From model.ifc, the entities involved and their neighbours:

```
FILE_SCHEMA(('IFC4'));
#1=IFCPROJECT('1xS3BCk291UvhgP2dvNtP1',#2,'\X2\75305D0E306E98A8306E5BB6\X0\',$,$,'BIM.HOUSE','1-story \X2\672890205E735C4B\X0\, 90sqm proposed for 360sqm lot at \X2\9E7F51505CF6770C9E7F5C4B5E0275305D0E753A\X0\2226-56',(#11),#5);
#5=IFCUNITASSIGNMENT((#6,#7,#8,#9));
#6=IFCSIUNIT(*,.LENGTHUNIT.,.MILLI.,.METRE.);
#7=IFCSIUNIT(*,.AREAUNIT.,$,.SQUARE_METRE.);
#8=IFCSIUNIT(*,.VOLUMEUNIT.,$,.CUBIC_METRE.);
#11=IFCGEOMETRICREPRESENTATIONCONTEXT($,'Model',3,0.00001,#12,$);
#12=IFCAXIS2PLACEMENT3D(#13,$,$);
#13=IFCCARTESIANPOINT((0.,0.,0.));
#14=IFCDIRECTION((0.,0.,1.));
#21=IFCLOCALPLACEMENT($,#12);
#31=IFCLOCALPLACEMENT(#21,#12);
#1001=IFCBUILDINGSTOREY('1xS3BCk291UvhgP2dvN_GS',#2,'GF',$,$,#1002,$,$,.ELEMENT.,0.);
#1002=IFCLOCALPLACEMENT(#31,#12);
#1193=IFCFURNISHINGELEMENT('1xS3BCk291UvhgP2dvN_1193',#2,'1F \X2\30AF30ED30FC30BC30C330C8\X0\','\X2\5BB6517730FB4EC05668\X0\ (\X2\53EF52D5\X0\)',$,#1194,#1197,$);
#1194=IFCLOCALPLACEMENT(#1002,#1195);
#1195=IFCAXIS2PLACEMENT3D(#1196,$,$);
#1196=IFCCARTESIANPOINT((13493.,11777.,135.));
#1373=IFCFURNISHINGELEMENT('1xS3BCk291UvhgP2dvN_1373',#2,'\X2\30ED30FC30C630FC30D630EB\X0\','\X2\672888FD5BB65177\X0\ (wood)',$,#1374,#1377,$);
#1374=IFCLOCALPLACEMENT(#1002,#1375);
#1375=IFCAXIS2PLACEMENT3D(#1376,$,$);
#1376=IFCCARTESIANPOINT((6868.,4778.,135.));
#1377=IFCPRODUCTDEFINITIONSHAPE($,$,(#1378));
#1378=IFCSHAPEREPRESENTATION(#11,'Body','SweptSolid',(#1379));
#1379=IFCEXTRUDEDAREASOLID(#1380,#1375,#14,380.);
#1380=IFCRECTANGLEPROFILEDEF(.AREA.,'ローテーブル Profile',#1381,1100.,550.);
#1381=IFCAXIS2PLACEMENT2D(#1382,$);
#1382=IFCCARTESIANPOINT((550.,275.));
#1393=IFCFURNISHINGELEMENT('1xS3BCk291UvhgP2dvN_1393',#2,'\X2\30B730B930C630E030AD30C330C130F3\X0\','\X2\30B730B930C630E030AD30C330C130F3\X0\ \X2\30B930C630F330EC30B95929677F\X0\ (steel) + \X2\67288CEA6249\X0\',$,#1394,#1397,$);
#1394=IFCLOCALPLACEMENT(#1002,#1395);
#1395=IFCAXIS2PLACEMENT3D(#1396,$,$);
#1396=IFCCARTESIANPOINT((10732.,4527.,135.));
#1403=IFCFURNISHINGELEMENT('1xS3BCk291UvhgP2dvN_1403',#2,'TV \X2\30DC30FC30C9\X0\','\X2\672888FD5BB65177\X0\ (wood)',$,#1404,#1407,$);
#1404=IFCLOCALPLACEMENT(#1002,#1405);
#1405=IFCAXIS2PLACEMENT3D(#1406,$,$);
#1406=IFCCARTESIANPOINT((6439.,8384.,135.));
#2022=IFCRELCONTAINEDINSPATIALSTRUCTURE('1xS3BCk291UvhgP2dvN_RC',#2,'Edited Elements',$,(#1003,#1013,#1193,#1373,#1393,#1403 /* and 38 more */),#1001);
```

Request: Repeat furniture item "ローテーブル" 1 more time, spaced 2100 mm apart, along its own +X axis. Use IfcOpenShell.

```python
import ifcopenshell
import ifcopenshell.api.geometry
import ifcopenshell.api.root
import ifcopenshell.util.element
import ifcopenshell.util.placement
import ifcopenshell.util.unit

model = ifcopenshell.open("model.ifc")
unit_scale = ifcopenshell.util.unit.calculate_unit_scale(model)


def reuse_history(source, copy):
    """copy_class also copies each property set's owner history, people and application; keep the originals."""
    for rel in copy.IsDefinedBy:
        if rel.is_a("IfcRelDefinesByProperties") and (history := rel.RelatingPropertyDefinition.OwnerHistory):
            rel.RelatingPropertyDefinition.OwnerHistory = source.OwnerHistory
            ifcopenshell.util.element.remove_deep2(model, history)


source = model.by_guid("1xS3BCk291UvhgP2dvN_1373")
base = ifcopenshell.util.placement.get_local_placement(source.ObjectPlacement)
step = base[:3, 0] * 2.1 / unit_scale

for i in range(1, 2):
    copy = ifcopenshell.api.root.copy_class(model, product=source)
    copy.Representation = ifcopenshell.util.element.copy_deep(
        model, source.Representation, exclude=["IfcGeometricRepresentationContext", "IfcRepresentationMap"]
    )
    reuse_history(source, copy)
    matrix = base.copy()
    matrix[:3, 3] += i * step
    print("added at", matrix[:3, 3].round(3) + 0.0)
    ifcopenshell.api.geometry.edit_object_placement(model, product=copy, matrix=matrix, is_si=False)

model.write("model-out.ifc")
```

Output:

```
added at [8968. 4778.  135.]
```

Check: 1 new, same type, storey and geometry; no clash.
